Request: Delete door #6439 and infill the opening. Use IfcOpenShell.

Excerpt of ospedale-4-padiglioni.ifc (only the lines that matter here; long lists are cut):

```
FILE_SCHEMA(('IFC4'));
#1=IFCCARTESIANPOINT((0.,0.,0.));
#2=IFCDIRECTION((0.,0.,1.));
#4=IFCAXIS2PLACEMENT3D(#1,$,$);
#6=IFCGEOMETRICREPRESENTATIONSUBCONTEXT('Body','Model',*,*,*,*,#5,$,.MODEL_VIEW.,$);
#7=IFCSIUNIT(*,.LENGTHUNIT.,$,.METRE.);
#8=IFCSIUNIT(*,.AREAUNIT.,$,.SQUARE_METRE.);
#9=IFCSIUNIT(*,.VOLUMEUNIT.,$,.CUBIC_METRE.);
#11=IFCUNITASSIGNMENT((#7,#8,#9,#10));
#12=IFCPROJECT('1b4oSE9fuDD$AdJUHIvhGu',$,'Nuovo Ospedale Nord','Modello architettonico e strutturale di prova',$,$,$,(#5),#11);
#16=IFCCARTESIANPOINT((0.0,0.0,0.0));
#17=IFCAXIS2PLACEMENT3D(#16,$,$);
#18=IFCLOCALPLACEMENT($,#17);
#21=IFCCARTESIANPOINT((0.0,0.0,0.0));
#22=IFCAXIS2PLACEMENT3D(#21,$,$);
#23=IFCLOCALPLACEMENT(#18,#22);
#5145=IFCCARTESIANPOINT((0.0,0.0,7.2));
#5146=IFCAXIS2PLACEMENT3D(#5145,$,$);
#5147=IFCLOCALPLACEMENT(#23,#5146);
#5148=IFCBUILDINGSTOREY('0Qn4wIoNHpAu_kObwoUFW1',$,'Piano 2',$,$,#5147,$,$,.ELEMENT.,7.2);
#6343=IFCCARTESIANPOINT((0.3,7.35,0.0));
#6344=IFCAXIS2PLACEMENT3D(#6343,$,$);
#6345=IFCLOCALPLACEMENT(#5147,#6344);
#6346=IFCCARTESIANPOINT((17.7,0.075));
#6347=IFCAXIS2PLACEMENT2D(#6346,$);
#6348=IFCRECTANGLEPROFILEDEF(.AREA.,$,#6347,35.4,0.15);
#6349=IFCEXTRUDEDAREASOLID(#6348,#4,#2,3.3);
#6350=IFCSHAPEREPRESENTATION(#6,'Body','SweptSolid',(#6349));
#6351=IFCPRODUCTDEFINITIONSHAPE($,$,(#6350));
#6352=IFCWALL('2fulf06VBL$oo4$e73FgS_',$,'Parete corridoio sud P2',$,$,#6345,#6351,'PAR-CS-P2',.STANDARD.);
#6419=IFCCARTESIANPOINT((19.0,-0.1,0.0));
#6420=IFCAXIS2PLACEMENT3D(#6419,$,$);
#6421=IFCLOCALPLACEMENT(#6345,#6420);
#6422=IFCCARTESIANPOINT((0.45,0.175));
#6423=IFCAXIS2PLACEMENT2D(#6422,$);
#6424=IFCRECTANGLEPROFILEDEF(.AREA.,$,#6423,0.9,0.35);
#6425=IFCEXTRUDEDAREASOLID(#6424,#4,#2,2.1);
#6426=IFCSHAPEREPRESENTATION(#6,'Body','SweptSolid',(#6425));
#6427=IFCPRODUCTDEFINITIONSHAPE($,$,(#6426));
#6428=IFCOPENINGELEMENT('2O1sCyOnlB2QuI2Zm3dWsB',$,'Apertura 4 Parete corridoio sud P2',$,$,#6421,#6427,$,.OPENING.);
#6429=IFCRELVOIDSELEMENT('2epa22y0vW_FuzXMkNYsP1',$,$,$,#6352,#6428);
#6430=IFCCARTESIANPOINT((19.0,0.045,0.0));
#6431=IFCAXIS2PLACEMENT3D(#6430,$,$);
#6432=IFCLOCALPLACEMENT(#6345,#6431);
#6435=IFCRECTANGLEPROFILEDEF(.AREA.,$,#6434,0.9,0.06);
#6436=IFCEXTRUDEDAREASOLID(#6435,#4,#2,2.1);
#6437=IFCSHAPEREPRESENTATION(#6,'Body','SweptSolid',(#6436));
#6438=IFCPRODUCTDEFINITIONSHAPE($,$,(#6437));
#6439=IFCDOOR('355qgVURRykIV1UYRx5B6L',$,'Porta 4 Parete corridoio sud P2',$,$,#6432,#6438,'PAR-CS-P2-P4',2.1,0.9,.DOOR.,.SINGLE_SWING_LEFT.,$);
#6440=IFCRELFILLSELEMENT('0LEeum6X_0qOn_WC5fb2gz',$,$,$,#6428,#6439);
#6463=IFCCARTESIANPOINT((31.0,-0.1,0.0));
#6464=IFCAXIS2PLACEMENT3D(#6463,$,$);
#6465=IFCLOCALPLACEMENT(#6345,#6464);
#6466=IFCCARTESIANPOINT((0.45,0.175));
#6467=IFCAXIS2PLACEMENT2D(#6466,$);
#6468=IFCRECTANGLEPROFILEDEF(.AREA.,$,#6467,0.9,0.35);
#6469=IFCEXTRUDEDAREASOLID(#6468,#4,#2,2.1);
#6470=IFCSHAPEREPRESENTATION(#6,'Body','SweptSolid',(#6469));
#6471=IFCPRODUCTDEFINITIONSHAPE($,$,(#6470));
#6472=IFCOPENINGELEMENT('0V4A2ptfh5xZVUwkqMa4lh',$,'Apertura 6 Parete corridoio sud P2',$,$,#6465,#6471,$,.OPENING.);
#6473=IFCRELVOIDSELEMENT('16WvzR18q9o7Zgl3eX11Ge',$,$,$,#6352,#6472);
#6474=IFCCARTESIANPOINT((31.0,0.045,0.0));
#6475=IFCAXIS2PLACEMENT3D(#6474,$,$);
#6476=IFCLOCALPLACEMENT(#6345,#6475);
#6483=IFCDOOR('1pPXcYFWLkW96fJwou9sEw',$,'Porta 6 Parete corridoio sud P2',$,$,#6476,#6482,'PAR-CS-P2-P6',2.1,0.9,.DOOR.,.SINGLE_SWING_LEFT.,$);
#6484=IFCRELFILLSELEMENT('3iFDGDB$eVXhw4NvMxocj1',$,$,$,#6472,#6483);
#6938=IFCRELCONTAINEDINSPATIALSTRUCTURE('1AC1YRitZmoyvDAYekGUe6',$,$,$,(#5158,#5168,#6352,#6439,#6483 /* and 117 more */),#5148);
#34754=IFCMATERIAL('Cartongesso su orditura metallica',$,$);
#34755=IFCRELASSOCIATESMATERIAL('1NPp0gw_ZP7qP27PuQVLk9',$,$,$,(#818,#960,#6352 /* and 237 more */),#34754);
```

```python
import ifcopenshell
import ifcopenshell.api.feature
import ifcopenshell.api.root
import ifcopenshell.geom
import ifcopenshell.util.shape

model = ifcopenshell.open("ospedale-4-padiglioni.ifc")
settings = ifcopenshell.geom.settings()


def volume(element):
    """Net volume in cubic metres, openings subtracted."""
    shape = ifcopenshell.geom.create_shape(settings, element)
    return ifcopenshell.util.shape.get_volume(shape.geometry)


door = model.by_guid("355qgVURRykIV1UYRx5B6L")
opening = door.FillsVoids[0].RelatingOpeningElement
wall = opening.VoidsElements[0].RelatingBuildingElement
before = volume(wall)

ifcopenshell.api.root.remove_product(model, product=door)
ifcopenshell.api.feature.remove_feature(model, feature=opening)

after = volume(wall)

print(f"wall volume {before:.3f} -> {after:.3f} m3")

model.write("ospedale-4-padiglioni-out.ifc")
```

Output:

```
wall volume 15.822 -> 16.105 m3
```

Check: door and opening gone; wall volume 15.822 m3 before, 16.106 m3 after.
